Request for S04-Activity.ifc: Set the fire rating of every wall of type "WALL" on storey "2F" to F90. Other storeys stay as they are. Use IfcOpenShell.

First a look at what the model holds.

```python
import ifcopenshell
import ifcopenshell.util.element

model = ifcopenshell.open("S04-Activity.ifc")
print(model.schema)
storey = next(s for s in model.by_type("IfcBuildingStorey") if s.Name == "2F")
walls = [e for e in ifcopenshell.util.element.get_decomposition(storey) if e.is_a("IfcWall")]
seen = {}
for e in walls:
    element_type = ifcopenshell.util.element.get_type(e)
    key = (element_type.Name if element_type != e and element_type else None, ifcopenshell.util.element.get_pset(e, "Pset_WallCommon", "FireRating"))
    seen[key] = seen.get(key, 0) + 1
for (name, value), count in sorted(seen.items(), key=str):
    print(count, "x", name, "|", value)
```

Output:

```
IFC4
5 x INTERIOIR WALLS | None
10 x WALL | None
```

```python
import ifcopenshell
import ifcopenshell.api.pset
import ifcopenshell.util.element

model = ifcopenshell.open("S04-Activity.ifc")

storey = next(s for s in model.by_type("IfcBuildingStorey") if s.Name == "2F")
walls = [e for e in ifcopenshell.util.element.get_decomposition(storey) if e.is_a("IfcWall")]

count = 0
for e in walls:
    element_type = ifcopenshell.util.element.get_type(e)
    if element_type in (None, e) or element_type.Name != "WALL":
        continue
    # add_pset returns the element's existing set when there is one.
    pset = ifcopenshell.api.pset.add_pset(model, product=e, name="Pset_WallCommon")
    ifcopenshell.api.pset.edit_pset(model, pset=pset, properties={"FireRating": "F90"})
    count += 1

print(count, "walls updated")

model.write("S04-Activity-out.ifc")
```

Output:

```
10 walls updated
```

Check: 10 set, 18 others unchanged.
